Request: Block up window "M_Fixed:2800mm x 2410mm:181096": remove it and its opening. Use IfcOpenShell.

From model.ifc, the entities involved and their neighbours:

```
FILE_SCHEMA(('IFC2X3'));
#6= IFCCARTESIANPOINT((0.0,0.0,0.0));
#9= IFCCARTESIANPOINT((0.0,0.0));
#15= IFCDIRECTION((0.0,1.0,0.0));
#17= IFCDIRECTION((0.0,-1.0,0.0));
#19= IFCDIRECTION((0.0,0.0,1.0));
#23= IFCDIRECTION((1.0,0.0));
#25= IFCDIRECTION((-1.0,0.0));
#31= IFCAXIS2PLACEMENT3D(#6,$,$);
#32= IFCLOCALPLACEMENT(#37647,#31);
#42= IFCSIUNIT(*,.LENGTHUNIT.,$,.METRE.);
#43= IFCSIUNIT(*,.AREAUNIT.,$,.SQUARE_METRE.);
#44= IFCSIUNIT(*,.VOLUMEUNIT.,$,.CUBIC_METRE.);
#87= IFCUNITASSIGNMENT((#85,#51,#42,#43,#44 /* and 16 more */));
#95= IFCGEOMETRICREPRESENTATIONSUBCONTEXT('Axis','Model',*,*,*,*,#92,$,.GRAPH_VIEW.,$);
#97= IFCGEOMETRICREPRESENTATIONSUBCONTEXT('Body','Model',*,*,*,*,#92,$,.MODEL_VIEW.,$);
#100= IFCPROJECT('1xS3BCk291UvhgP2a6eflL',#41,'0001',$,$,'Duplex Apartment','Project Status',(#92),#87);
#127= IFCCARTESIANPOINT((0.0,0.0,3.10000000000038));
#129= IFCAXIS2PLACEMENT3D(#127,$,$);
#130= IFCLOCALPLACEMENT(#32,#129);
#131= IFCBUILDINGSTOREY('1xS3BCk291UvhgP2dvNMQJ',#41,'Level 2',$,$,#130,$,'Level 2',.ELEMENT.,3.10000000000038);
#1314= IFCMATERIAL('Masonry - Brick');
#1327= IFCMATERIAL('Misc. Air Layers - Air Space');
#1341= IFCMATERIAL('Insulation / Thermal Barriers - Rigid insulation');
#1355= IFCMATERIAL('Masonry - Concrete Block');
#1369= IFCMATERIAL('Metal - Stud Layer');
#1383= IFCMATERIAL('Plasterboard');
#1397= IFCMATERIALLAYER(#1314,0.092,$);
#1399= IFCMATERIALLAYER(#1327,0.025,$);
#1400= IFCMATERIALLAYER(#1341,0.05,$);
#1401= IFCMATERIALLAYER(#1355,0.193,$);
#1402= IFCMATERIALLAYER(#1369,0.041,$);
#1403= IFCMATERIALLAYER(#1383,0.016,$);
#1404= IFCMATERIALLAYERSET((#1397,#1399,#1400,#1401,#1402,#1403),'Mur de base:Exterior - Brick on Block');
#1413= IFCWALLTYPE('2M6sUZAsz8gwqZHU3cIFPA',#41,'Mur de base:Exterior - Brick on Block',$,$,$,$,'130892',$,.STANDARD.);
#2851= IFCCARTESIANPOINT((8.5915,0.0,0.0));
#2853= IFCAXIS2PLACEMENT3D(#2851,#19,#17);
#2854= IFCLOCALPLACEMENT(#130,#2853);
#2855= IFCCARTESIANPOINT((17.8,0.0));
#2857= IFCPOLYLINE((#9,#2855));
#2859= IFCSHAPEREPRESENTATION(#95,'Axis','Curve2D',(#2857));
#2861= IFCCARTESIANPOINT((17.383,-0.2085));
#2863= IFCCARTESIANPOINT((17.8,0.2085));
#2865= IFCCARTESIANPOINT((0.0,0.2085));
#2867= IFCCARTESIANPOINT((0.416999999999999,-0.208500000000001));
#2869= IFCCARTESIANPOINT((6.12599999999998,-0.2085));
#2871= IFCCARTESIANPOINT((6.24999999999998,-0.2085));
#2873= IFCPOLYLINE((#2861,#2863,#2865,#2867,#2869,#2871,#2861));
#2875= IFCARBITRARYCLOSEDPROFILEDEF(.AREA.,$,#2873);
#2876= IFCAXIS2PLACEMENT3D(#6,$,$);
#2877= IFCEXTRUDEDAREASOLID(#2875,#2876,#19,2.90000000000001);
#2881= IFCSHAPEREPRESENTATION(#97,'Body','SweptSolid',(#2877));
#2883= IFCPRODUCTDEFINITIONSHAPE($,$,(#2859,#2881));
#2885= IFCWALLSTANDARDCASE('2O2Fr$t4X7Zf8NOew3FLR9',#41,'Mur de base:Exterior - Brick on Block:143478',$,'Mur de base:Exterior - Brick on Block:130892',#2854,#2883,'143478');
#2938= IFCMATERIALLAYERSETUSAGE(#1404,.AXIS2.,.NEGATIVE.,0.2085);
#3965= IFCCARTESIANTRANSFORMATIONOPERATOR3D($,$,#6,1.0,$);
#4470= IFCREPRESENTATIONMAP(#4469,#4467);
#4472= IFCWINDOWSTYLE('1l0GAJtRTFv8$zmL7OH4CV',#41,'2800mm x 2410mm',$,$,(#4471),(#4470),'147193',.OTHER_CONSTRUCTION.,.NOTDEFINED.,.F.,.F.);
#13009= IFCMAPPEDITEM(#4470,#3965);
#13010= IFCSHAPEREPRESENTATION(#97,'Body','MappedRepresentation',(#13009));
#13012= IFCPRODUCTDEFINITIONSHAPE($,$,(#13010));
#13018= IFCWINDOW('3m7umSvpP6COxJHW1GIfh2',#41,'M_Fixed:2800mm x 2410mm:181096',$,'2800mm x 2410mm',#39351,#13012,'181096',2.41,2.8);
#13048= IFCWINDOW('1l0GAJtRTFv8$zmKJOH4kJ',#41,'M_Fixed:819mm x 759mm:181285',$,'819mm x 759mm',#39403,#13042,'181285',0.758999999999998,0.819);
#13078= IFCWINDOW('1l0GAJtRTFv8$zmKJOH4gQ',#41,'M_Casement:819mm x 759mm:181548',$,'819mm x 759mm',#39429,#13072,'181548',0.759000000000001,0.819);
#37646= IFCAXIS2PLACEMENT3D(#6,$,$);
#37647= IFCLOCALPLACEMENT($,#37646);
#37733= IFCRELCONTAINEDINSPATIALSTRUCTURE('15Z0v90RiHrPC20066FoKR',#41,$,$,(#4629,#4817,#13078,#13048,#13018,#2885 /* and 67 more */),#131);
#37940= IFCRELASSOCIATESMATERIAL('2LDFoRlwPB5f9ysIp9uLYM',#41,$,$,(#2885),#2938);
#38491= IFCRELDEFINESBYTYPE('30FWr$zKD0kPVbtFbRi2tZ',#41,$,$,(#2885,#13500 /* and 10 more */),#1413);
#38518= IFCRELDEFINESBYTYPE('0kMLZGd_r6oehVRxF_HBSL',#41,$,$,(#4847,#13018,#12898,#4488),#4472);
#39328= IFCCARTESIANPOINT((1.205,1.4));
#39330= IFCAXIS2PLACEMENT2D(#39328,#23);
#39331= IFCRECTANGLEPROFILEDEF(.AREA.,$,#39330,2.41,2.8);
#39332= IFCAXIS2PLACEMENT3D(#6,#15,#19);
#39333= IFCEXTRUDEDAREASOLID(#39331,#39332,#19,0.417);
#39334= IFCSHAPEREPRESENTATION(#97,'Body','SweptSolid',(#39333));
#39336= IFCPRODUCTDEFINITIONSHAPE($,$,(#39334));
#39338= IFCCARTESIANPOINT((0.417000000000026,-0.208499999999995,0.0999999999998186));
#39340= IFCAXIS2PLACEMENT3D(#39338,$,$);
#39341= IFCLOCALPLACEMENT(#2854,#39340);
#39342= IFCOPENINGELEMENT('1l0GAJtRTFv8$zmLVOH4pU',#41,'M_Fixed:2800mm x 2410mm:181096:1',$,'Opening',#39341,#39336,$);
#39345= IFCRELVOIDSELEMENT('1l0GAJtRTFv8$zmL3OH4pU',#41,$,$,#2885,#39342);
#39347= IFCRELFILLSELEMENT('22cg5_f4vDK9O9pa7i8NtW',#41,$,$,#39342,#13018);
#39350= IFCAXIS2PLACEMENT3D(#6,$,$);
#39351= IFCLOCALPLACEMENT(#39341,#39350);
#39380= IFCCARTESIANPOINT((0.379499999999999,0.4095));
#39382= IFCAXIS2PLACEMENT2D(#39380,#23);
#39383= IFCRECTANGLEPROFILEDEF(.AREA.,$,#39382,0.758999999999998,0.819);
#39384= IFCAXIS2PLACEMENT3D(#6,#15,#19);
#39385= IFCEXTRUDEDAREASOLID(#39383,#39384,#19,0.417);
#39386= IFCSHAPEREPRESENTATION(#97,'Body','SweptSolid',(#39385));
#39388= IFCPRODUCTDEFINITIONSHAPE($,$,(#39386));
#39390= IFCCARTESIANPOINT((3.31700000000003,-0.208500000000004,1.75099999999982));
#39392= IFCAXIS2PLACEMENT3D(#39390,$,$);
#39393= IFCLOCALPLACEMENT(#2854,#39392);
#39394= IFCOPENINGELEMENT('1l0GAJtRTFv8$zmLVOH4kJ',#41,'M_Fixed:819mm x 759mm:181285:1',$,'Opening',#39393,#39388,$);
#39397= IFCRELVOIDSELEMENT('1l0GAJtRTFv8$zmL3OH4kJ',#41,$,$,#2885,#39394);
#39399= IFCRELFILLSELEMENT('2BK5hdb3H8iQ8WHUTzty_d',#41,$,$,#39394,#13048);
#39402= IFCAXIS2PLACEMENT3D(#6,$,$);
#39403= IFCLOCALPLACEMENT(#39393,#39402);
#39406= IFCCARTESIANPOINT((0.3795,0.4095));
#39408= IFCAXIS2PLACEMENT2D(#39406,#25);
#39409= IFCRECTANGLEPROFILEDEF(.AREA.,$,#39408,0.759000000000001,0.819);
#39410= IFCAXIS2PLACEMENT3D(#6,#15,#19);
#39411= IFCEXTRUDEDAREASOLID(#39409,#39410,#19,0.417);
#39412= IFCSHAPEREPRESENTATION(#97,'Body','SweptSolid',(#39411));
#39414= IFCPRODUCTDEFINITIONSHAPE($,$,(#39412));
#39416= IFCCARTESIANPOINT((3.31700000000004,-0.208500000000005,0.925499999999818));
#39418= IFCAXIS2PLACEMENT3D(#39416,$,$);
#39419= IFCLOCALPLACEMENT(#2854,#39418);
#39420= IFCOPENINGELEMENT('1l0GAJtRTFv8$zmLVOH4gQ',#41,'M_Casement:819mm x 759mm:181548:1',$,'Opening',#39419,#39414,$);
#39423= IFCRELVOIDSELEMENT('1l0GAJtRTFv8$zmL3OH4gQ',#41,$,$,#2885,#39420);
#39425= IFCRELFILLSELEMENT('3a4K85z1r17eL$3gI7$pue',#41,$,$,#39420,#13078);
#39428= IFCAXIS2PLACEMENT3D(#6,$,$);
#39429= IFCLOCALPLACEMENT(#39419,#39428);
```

```python
import ifcopenshell
import ifcopenshell.api.feature
import ifcopenshell.api.root
import ifcopenshell.geom
import ifcopenshell.util.shape

model = ifcopenshell.open("model.ifc")
settings = ifcopenshell.geom.settings()


def volume(element):
    """Net volume in cubic metres, openings subtracted."""
    shape = ifcopenshell.geom.create_shape(settings, element)
    return ifcopenshell.util.shape.get_volume(shape.geometry)


window = model.by_guid("3m7umSvpP6COxJHW1GIfh2")
opening = window.FillsVoids[0].RelatingOpeningElement
wall = opening.VoidsElements[0].RelatingBuildingElement
before = volume(wall)

ifcopenshell.api.root.remove_product(model, product=window)
ifcopenshell.api.feature.remove_feature(model, feature=opening)

after = volume(wall)

print(f"wall volume {before:.3f} -> {after:.3f} m3")

model.write("model_v2.ifc")
```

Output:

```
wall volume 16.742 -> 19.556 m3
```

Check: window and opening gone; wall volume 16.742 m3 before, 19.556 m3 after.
